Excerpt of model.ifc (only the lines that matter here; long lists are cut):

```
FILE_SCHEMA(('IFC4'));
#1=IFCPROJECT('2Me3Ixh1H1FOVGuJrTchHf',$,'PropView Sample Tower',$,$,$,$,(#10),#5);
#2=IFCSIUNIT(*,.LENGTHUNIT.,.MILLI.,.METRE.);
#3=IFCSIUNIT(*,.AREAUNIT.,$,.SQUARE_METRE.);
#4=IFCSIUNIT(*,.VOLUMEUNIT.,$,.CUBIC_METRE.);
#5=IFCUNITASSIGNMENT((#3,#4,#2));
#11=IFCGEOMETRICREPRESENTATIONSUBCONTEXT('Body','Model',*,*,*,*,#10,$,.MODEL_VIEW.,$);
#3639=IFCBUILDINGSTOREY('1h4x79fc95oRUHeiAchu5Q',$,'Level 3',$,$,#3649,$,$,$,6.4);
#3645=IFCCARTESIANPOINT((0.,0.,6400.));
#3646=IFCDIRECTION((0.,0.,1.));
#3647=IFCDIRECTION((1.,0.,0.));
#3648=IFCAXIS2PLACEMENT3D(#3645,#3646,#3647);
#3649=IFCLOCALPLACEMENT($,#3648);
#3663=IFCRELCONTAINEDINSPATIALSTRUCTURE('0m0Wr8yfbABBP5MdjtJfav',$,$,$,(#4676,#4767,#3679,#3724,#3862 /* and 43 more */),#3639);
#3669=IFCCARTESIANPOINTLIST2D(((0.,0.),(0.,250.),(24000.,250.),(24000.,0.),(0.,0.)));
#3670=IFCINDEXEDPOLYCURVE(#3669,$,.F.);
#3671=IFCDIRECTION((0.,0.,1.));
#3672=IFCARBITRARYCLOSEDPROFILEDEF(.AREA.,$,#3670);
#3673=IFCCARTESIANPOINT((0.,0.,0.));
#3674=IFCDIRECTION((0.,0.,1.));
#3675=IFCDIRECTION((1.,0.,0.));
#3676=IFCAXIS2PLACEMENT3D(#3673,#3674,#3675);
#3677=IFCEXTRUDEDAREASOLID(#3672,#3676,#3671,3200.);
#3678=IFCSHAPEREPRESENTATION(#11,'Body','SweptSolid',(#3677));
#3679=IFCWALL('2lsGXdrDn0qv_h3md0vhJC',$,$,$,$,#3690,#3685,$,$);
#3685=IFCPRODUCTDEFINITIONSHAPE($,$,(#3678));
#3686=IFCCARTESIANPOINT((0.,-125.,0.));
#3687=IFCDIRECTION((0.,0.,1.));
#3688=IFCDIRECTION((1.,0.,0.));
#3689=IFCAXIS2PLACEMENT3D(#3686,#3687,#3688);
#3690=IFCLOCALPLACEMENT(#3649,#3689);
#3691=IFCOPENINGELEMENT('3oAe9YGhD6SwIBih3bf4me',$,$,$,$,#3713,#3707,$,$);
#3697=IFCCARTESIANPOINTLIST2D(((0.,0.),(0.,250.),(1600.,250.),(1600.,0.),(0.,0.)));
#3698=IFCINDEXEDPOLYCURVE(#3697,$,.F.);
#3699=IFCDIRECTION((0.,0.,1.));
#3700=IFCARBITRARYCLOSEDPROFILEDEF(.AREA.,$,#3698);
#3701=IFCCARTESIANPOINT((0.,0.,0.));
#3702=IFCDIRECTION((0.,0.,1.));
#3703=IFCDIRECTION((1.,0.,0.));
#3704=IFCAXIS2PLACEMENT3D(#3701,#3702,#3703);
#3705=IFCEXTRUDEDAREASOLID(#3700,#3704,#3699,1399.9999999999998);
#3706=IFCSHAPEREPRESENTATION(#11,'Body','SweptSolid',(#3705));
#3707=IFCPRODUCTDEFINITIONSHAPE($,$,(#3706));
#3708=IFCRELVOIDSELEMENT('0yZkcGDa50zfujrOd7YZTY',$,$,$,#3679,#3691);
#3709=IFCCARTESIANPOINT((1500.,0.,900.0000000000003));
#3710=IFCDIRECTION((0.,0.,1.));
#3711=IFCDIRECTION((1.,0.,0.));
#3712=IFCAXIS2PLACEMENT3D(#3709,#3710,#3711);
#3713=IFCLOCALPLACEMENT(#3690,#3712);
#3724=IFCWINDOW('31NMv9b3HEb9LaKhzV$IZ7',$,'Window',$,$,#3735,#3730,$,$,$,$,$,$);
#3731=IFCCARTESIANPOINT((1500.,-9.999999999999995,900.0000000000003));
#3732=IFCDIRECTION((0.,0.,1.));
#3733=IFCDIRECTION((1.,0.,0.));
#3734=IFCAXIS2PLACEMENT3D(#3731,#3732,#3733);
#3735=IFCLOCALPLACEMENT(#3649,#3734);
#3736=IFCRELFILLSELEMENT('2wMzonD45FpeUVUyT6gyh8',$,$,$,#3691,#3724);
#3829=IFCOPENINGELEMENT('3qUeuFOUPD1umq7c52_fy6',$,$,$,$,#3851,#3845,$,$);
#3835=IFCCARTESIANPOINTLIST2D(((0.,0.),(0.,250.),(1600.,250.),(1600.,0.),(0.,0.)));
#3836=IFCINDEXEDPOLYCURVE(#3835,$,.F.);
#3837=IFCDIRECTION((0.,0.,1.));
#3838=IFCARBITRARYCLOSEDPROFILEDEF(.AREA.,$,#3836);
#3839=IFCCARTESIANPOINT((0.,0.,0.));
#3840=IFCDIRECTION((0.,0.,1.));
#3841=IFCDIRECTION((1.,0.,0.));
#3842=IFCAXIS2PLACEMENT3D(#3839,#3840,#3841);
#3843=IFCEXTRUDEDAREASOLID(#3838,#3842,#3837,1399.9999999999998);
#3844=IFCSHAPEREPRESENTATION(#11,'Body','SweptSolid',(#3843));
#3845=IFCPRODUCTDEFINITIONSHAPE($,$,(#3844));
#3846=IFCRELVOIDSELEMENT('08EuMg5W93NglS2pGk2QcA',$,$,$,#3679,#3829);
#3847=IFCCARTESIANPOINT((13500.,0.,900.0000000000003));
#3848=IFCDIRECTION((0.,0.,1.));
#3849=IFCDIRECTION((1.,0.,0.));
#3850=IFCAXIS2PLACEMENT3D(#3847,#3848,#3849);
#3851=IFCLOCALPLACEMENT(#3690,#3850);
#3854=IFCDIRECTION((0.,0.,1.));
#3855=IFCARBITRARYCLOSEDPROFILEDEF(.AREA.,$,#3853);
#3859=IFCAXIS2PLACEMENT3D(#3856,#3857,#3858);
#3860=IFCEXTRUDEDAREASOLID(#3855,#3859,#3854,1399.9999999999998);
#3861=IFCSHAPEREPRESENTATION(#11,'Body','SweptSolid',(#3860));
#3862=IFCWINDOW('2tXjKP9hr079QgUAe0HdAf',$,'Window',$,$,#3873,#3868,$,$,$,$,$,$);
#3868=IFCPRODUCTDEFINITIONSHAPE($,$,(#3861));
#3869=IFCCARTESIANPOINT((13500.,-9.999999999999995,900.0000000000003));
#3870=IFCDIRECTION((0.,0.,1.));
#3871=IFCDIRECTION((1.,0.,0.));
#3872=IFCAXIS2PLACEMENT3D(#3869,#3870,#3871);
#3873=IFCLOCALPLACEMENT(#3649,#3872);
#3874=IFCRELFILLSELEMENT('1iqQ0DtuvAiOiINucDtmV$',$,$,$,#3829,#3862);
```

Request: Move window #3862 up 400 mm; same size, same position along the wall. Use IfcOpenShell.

```python
import numpy as np
import ifcopenshell
import ifcopenshell.api.geometry
import ifcopenshell.util.placement
import ifcopenshell.util.unit

model = ifcopenshell.open("model.ifc")
unit_scale = ifcopenshell.util.unit.calculate_unit_scale(model)

window = model.by_id(3862)
opening = window.FillsVoids[0].RelatingOpeningElement
dz = 0.4 / unit_scale

shift = np.array([0.0, 0.0, dz])
# The window is not placed relative to its opening, so move both.
for product in (opening, window):
    matrix = ifcopenshell.util.placement.get_local_placement(product.ObjectPlacement)
    matrix[:3, 3] += shift
    ifcopenshell.api.geometry.edit_object_placement(model, product=product, matrix=matrix, is_si=False)

print(f"moved by {dz * unit_scale:+.3f} m")

model.write("model_rev.ifc")
```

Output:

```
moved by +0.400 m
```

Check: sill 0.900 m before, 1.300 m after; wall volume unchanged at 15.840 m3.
